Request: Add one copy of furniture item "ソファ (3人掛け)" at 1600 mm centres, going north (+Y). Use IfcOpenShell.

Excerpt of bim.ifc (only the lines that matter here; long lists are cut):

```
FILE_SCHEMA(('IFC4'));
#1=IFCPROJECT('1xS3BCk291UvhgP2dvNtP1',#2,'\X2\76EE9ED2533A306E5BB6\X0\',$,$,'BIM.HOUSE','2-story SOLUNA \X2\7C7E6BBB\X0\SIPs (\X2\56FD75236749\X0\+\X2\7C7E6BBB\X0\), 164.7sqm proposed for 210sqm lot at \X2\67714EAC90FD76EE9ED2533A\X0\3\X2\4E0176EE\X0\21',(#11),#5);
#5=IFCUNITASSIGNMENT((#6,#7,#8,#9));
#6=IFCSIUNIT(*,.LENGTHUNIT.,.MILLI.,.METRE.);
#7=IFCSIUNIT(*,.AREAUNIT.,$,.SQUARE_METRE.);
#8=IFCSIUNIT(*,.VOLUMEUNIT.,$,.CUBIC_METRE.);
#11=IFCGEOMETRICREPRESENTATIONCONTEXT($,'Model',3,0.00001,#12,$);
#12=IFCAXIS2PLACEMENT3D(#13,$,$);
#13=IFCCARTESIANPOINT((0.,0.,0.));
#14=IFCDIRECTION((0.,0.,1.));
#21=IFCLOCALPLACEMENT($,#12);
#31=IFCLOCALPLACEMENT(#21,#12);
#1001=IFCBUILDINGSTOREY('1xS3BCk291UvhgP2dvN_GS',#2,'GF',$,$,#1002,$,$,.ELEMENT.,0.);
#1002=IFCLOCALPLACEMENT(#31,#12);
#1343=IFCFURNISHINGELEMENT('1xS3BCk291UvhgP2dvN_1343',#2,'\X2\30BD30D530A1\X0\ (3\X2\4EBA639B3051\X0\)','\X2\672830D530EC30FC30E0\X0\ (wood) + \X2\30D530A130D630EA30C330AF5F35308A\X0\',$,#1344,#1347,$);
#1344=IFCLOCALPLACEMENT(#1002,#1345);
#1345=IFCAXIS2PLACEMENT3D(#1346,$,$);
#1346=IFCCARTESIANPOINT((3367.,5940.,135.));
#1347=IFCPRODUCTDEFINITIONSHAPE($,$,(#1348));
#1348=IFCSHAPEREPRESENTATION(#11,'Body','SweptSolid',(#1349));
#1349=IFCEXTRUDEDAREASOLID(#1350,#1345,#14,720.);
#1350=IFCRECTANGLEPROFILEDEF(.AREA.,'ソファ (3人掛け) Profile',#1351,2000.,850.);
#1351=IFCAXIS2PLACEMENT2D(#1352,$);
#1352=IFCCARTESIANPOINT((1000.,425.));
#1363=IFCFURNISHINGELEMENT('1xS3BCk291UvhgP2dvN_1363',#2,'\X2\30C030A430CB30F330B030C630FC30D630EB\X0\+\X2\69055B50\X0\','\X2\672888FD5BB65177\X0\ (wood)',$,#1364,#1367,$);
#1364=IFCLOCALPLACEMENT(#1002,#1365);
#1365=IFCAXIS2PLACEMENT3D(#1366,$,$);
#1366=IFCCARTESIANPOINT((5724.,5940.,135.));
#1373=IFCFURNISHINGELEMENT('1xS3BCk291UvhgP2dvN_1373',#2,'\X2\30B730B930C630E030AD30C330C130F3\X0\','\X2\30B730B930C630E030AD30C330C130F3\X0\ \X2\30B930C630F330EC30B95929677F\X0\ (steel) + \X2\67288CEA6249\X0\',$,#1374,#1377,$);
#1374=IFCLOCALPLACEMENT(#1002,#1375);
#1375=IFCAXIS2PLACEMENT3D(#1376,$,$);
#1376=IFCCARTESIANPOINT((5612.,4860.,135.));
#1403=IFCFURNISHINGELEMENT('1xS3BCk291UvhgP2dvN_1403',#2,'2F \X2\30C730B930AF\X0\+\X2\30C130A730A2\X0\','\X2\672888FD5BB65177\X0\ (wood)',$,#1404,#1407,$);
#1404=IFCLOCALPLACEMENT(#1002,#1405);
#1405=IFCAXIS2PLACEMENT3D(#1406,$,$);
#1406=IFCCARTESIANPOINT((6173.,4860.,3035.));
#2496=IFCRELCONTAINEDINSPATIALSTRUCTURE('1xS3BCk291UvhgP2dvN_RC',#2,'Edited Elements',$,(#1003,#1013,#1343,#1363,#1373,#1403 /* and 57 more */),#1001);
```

```python
import numpy as np
import ifcopenshell
import ifcopenshell.api.geometry
import ifcopenshell.api.root
import ifcopenshell.util.element
import ifcopenshell.util.placement
import ifcopenshell.util.unit

model = ifcopenshell.open("bim.ifc")
unit_scale = ifcopenshell.util.unit.calculate_unit_scale(model)


def reuse_history(source, copy):
    """copy_class also copies each property set's owner history, people and application; keep the originals."""
    for rel in copy.IsDefinedBy:
        if rel.is_a("IfcRelDefinesByProperties") and (history := rel.RelatingPropertyDefinition.OwnerHistory):
            rel.RelatingPropertyDefinition.OwnerHistory = source.OwnerHistory
            ifcopenshell.util.element.remove_deep2(model, history)


source = model.by_guid("1xS3BCk291UvhgP2dvN_1343")
base = ifcopenshell.util.placement.get_local_placement(source.ObjectPlacement)
step = np.array([0.0, 1.0, 0.0]) * 1.6 / unit_scale

for i in range(1, 2):
    copy = ifcopenshell.api.root.copy_class(model, product=source)
    copy.Representation = ifcopenshell.util.element.copy_deep(
        model, source.Representation, exclude=["IfcGeometricRepresentationContext", "IfcRepresentationMap"]
    )
    reuse_history(source, copy)
    matrix = base.copy()
    matrix[:3, 3] += i * step
    print("added at", matrix[:3, 3].round(3) + 0.0)
    ifcopenshell.api.geometry.edit_object_placement(model, product=copy, matrix=matrix, is_si=False)

model.write("bim_rev.ifc")
```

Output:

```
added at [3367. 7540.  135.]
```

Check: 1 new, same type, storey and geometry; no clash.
